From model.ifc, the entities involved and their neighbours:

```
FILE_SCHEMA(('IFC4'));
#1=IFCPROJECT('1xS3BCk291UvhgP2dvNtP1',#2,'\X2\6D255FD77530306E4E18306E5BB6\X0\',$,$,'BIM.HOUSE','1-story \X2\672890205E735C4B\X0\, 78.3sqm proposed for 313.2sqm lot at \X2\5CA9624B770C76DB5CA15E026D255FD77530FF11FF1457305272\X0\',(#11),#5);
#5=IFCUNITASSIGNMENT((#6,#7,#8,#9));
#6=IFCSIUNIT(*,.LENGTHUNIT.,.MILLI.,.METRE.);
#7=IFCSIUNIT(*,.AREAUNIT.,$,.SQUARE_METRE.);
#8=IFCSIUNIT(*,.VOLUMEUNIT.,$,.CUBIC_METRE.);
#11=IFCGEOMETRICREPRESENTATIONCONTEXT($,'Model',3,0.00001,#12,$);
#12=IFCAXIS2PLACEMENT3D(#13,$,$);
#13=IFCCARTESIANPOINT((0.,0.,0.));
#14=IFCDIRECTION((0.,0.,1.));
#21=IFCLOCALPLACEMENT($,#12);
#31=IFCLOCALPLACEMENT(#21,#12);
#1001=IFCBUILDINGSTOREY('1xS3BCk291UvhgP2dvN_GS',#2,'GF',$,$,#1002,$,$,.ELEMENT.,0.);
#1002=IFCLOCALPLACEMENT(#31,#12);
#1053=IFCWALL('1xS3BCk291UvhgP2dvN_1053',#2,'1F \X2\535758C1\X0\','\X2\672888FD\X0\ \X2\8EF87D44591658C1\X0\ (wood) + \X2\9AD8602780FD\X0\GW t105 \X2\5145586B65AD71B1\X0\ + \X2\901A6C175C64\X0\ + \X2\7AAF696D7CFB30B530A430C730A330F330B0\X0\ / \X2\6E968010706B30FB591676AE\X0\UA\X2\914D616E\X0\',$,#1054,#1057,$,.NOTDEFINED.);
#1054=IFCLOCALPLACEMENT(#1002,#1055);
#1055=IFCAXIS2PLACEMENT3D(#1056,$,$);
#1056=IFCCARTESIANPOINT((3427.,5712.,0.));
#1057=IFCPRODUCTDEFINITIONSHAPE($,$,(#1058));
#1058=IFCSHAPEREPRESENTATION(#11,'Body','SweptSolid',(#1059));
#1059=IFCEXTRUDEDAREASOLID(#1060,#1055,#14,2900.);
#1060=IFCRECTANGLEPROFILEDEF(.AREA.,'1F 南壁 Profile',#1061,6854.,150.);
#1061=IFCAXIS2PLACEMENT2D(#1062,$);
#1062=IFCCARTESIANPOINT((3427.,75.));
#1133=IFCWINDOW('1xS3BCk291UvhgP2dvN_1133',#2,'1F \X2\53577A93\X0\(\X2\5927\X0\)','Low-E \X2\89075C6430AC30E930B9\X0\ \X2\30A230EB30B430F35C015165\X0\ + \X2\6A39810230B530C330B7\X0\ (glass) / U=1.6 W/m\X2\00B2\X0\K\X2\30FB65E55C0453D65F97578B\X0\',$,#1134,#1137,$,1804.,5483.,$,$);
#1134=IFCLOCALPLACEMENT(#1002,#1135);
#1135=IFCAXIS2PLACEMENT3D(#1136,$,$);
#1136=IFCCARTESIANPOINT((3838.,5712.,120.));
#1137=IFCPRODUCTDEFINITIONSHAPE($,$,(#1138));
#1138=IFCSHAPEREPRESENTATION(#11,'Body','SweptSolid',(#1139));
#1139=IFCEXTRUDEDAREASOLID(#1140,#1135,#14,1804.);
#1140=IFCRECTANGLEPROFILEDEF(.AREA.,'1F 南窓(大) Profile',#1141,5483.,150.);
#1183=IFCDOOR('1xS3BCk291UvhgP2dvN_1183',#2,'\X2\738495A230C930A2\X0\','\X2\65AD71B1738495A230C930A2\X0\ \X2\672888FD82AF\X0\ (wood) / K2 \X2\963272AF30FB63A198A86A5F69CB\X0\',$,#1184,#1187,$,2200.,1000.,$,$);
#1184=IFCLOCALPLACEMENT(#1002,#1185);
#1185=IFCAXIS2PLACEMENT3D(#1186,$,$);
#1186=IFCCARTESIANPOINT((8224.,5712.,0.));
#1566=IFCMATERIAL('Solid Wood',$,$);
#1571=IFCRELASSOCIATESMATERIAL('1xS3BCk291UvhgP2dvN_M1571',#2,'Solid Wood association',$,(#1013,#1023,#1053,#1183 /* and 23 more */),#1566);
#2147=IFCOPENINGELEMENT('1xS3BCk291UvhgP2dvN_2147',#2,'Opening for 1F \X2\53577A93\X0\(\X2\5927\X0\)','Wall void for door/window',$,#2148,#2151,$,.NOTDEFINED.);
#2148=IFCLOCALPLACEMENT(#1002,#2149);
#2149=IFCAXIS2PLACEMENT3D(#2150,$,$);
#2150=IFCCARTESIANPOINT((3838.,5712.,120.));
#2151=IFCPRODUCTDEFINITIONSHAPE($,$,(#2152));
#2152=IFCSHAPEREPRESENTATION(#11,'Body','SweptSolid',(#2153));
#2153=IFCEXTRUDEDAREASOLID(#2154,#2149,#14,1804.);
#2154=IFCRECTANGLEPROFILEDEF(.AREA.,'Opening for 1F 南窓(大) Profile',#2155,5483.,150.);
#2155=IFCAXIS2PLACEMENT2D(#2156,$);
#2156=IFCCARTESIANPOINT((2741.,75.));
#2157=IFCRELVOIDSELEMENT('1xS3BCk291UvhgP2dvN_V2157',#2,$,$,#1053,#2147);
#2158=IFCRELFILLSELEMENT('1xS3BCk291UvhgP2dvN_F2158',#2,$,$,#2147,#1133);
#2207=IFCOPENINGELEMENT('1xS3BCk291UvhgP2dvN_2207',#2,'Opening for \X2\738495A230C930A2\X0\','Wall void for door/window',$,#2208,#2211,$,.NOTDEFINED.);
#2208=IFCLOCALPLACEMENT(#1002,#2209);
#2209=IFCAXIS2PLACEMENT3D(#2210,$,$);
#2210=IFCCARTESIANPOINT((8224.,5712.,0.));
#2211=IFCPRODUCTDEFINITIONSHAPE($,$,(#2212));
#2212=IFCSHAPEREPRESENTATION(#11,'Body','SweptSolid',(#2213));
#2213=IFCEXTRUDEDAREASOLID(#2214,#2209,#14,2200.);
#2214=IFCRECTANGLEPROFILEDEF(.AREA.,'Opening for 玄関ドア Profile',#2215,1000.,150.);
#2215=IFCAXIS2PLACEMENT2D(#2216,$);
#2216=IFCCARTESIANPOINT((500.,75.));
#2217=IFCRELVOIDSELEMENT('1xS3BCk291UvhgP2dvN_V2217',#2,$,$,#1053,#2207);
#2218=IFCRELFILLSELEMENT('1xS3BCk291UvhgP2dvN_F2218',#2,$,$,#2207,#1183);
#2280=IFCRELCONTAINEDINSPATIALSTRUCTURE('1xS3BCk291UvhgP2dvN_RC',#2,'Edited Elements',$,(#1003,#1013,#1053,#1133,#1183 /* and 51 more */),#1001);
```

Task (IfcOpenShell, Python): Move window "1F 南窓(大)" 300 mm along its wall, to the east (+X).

```python
import ifcopenshell
import ifcopenshell.api.geometry
import ifcopenshell.util.placement

model = ifcopenshell.open("model.ifc")

window = model.by_guid("1xS3BCk291UvhgP2dvN_1133")
opening = window.FillsVoids[0].RelatingOpeningElement
wall = opening.VoidsElements[0].RelatingBuildingElement

wall_matrix = ifcopenshell.util.placement.get_local_placement(wall.ObjectPlacement)
shift = wall_matrix[:3, 0] * 300.0
before = ifcopenshell.util.placement.get_local_placement(window.ObjectPlacement)[:3, 3].copy()

# The window is not placed relative to its opening, so move both.
for product in (opening, window):
    matrix = ifcopenshell.util.placement.get_local_placement(product.ObjectPlacement)
    matrix[:3, 3] += shift
    ifcopenshell.api.geometry.edit_object_placement(model, product=product, matrix=matrix, is_si=False)

after = ifcopenshell.util.placement.get_local_placement(window.ObjectPlacement)[:3, 3]
print("window moved by", (after - before).round(3) + 0.0)

model.write("model-out.ifc")
```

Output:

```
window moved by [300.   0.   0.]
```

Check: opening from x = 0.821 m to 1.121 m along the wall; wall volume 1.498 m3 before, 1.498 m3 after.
